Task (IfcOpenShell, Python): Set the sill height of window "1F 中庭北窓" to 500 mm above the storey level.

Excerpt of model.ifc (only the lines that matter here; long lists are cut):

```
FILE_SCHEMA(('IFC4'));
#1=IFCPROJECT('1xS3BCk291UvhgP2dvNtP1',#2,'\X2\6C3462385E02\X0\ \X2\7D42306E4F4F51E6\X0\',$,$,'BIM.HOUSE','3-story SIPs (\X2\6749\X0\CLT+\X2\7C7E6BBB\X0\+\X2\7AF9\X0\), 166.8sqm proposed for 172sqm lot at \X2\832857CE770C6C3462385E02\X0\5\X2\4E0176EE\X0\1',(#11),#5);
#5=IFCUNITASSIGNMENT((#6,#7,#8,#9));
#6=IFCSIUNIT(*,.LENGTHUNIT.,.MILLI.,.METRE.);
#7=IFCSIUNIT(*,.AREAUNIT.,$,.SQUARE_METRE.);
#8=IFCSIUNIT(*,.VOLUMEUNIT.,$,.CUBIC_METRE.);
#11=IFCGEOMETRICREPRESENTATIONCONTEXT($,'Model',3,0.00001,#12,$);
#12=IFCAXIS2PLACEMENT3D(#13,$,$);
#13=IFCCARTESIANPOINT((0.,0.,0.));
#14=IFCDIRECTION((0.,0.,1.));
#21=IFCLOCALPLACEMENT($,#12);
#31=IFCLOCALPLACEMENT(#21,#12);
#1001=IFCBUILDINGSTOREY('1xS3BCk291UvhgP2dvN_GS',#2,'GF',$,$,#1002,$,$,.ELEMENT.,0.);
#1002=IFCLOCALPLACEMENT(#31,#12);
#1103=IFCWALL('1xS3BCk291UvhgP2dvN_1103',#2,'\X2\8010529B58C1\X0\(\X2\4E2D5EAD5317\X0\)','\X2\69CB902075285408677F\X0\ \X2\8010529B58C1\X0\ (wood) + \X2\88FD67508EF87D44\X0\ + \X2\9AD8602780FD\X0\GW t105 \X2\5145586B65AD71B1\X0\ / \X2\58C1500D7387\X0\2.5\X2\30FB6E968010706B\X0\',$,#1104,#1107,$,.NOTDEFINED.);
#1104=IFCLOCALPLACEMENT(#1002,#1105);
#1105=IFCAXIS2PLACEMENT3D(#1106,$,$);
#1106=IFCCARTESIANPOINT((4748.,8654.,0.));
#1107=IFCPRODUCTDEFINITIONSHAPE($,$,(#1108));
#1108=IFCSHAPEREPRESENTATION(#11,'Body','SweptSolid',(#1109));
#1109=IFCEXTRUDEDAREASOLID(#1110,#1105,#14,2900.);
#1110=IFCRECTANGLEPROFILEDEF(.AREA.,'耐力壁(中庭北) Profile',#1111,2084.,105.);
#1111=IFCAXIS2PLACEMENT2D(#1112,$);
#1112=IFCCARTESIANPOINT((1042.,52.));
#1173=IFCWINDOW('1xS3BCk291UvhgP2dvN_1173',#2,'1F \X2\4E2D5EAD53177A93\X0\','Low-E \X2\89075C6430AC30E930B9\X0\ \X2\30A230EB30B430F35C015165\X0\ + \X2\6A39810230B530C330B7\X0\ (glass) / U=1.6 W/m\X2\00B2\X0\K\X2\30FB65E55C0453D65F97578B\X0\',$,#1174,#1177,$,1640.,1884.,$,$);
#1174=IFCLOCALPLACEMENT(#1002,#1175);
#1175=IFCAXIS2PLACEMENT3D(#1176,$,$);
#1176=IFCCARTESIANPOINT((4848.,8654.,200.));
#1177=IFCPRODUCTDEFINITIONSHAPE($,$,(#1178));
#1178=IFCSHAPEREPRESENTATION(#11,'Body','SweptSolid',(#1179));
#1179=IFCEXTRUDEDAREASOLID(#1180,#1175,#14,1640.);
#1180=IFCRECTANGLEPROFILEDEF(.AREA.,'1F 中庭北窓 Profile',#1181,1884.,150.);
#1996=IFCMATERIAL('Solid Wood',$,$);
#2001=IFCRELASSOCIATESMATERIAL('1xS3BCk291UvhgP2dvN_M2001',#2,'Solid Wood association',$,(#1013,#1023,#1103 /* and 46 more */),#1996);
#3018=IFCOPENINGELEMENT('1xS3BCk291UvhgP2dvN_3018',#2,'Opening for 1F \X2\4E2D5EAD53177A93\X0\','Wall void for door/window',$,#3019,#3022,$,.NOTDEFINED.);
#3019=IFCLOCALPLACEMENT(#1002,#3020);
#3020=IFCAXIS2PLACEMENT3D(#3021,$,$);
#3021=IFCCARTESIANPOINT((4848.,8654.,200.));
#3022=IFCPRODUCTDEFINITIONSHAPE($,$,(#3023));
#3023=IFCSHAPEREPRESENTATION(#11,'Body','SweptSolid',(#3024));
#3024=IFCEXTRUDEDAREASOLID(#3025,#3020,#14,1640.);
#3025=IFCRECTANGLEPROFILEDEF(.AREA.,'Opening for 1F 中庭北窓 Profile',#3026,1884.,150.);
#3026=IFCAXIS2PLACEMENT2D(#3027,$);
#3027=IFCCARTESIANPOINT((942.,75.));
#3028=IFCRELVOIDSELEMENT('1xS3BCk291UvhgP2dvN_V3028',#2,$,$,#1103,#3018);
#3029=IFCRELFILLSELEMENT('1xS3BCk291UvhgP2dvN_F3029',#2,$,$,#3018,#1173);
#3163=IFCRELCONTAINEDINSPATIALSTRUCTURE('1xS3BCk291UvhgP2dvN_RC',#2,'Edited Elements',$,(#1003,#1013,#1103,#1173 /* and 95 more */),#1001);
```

```python
import numpy as np
import ifcopenshell
import ifcopenshell.api.geometry
import ifcopenshell.geom
import ifcopenshell.util.element
import ifcopenshell.util.placement
import ifcopenshell.util.shape
import ifcopenshell.util.unit

model = ifcopenshell.open("model.ifc")
unit_scale = ifcopenshell.util.unit.calculate_unit_scale(model)

window = model.by_guid("1xS3BCk291UvhgP2dvN_1173")
opening = window.FillsVoids[0].RelatingOpeningElement
storey = ifcopenshell.util.element.get_container(window, ifc_class="IfcBuildingStorey")
level = ifcopenshell.util.placement.get_local_placement(storey.ObjectPlacement)[2, 3]

# The opening's origin need not be at the sill, so measure its lowest point.
shape = ifcopenshell.geom.create_shape(ifcopenshell.geom.settings(), opening)
bottom = ifcopenshell.util.shape.get_shape_bottom_elevation(shape, shape.geometry) / unit_scale
dz = level + 0.5 / unit_scale - bottom

shift = np.array([0.0, 0.0, dz])
# The window is not placed relative to its opening, so move both.
for product in (opening, window):
    matrix = ifcopenshell.util.placement.get_local_placement(product.ObjectPlacement)
    matrix[:3, 3] += shift
    ifcopenshell.api.geometry.edit_object_placement(model, product=product, matrix=matrix, is_si=False)

print(f"moved by {dz * unit_scale:+.3f} m")

model.write("model_rev.ifc")
```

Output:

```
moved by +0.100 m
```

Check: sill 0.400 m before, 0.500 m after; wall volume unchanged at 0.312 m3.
